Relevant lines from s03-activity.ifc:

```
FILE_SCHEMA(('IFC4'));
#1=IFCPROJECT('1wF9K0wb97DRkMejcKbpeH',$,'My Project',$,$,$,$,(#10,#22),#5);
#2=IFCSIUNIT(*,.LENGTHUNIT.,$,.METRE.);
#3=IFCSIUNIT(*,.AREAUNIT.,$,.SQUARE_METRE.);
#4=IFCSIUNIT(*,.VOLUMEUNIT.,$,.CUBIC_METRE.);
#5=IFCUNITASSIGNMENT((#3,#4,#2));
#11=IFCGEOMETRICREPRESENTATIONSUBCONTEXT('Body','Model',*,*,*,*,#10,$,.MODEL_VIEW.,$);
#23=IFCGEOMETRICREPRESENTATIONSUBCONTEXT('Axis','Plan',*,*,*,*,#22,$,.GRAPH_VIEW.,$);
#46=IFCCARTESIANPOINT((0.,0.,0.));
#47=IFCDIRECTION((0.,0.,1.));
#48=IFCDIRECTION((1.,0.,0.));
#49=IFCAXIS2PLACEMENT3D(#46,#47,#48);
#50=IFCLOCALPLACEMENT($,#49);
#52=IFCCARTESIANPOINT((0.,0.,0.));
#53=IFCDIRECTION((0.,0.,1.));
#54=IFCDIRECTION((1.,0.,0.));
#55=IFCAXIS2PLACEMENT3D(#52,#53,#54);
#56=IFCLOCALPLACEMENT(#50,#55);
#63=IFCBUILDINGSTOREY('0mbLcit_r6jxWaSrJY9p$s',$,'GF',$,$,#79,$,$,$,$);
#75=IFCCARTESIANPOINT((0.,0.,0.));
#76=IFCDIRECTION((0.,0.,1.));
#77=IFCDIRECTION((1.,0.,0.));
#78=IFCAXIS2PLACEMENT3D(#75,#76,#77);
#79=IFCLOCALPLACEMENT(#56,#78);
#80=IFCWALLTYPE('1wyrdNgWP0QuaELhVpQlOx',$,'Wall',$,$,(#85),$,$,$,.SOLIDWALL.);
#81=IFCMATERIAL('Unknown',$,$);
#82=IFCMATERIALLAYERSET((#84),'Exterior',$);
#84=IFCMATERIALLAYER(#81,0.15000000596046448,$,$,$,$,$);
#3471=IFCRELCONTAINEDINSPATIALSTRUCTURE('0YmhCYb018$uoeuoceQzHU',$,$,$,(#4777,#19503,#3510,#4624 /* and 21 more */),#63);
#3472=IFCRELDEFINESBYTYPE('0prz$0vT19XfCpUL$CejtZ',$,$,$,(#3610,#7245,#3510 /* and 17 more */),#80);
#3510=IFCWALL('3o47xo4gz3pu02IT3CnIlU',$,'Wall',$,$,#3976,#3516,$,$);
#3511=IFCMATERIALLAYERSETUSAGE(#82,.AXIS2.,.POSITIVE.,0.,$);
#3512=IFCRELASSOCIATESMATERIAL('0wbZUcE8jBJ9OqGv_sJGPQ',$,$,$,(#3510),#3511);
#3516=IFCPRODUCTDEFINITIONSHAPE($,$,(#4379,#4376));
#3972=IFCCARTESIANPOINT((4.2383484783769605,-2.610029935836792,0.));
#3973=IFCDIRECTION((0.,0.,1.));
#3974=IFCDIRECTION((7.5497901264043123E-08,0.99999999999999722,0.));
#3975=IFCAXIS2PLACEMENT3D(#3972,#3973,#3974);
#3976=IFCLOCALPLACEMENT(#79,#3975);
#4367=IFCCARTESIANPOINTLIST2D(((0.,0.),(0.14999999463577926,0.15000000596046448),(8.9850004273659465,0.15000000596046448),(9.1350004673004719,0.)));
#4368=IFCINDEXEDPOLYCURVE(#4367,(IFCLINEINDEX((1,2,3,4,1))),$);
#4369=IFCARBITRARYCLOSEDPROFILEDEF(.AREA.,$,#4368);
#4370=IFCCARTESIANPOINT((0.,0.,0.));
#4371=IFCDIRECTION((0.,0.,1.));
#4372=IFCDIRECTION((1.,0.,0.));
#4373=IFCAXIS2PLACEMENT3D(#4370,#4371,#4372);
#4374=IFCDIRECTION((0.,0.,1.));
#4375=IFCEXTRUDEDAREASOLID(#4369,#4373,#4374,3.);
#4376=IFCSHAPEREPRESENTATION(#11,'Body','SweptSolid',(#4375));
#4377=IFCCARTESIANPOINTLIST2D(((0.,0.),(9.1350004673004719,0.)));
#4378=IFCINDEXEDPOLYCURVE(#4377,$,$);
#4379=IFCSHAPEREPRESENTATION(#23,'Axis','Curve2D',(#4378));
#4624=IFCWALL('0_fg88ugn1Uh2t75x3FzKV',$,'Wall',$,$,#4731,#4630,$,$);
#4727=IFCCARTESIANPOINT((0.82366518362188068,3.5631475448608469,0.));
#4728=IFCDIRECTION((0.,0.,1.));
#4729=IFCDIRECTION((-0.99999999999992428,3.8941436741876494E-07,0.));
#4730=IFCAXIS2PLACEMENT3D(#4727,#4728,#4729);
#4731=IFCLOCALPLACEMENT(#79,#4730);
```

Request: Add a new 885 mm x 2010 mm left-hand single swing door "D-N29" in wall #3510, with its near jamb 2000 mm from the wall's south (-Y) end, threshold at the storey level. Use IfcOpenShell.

```python
import numpy as np
import ifcopenshell
import ifcopenshell.api.feature
import ifcopenshell.api.geometry
import ifcopenshell.api.root
import ifcopenshell.api.spatial
import ifcopenshell.geom
import ifcopenshell.util.element
import ifcopenshell.util.placement
import ifcopenshell.util.representation
import ifcopenshell.util.shape
import ifcopenshell.util.unit

model = ifcopenshell.open("s03-activity.ifc")
unit_scale = ifcopenshell.util.unit.calculate_unit_scale(model)
settings = ifcopenshell.geom.settings()


def volume(element):
    """Net volume in cubic metres, openings subtracted."""
    shape = ifcopenshell.geom.create_shape(settings, element)
    return ifcopenshell.util.shape.get_volume(shape.geometry)


wall = model.by_id(3510)
storey = ifcopenshell.util.element.get_container(wall, ifc_class="IfcBuildingStorey")
context = ifcopenshell.util.representation.get_context(model, "Model", "Body", "MODEL_VIEW")
before = volume(wall)

width, height, from_end, sill = 0.885, 2.01, 2, 0.0  # metres

# The wall runs along its own X axis, and the end named is its -X end.
wall_shape = ifcopenshell.geom.create_shape(settings, wall)
x, y, z = ifcopenshell.util.shape.get_vertices(wall_shape.geometry).T
start = x.min() + from_end
face, thickness = float(y.min()), float(y.max() - y.min())
wall_matrix = ifcopenshell.util.placement.get_local_placement(wall.ObjectPlacement)
level = ifcopenshell.util.placement.get_local_placement(storey.ObjectPlacement)[2, 3]


def in_wall(x, y):
    """Placement at x, y metres in the wall's axes, at sill height."""
    matrix = wall_matrix.copy()
    matrix[:, 3] = wall_matrix @ np.array([x / unit_scale, y / unit_scale, 0.0, 1.0])
    matrix[2, 3] = level + sill / unit_scale
    return matrix


# Opening: a box that overshoots both wall faces by 50 mm.
opening = ifcopenshell.api.root.create_entity(model, ifc_class="IfcOpeningElement", predefined_type="OPENING")
box = ifcopenshell.api.geometry.add_wall_representation(
    model, context=context, length=width, height=height, thickness=thickness + 0.1
)
ifcopenshell.api.geometry.assign_representation(model, product=opening, representation=box)
ifcopenshell.api.geometry.edit_object_placement(model, product=opening, matrix=in_wall(start, face - 0.05), is_si=False)
ifcopenshell.api.feature.add_feature(model, feature=opening, element=wall)

door = ifcopenshell.api.root.create_entity(model, ifc_class="IfcDoor", name="D-N29", predefined_type="DOOR")
door.OverallWidth, door.OverallHeight = width / unit_scale, height / unit_scale
door.OperationType = "SINGLE_SWING_LEFT"
body = ifcopenshell.api.geometry.add_door_representation(
    model,
    context=context,
    overall_width=door.OverallWidth,
    overall_height=door.OverallHeight,
    operation_type="SINGLE_SWING_LEFT",
    lining_properties={"LiningDepth": thickness / unit_scale, "ThresholdDepth": thickness / unit_scale},
)
ifcopenshell.api.geometry.assign_representation(model, product=door, representation=body)
ifcopenshell.api.spatial.assign_container(model, products=[door], relating_structure=storey)
ifcopenshell.api.feature.add_filling(model, opening=opening, element=door)

# The lining spans the wall, so the door starts at the wall face.
ifcopenshell.api.geometry.edit_object_placement(model, product=door, matrix=in_wall(start, face), is_si=False)

after = volume(wall)

print(f"wall volume {before:.3f} -> {after:.3f} m3")

model.write("s03-activity_v2.ifc")
```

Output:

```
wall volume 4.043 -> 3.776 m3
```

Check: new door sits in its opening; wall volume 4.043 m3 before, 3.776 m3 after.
